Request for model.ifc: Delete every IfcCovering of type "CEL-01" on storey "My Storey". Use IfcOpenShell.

First a look at what the model holds.

```python
import ifcopenshell
import ifcopenshell.util.element

model = ifcopenshell.open("model.ifc")
print(model.schema)
storey = next(s for s in model.by_type("IfcBuildingStorey") if s.Name == "My Storey")
coverings = [e for e in ifcopenshell.util.element.get_decomposition(storey) if e.is_a("IfcCovering")]
seen = {}
for e in coverings:
    element_type = ifcopenshell.util.element.get_type(e)
    name = element_type.Name if element_type not in (None, e) else None
    seen[name] = seen.get(name, 0) + 1
for name, count in sorted(seen.items(), key=str):
    print(count, "x", name)
```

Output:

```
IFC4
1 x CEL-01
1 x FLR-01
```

```python
import ifcopenshell
import ifcopenshell.api.root
import ifcopenshell.util.element

model = ifcopenshell.open("model.ifc")

storey = next(s for s in model.by_type("IfcBuildingStorey") if s.Name == "My Storey")
coverings = [e for e in ifcopenshell.util.element.get_decomposition(storey) if e.is_a("IfcCovering")]
targets = [e for e in coverings if (t := ifcopenshell.util.element.get_type(e)) not in (None, e) and t.Name == "CEL-01"]

for e in targets:
    ifcopenshell.api.root.remove_product(model, product=e)
print(len(targets), "removed")

model.write("model_updated.ifc")
```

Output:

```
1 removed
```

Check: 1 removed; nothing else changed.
